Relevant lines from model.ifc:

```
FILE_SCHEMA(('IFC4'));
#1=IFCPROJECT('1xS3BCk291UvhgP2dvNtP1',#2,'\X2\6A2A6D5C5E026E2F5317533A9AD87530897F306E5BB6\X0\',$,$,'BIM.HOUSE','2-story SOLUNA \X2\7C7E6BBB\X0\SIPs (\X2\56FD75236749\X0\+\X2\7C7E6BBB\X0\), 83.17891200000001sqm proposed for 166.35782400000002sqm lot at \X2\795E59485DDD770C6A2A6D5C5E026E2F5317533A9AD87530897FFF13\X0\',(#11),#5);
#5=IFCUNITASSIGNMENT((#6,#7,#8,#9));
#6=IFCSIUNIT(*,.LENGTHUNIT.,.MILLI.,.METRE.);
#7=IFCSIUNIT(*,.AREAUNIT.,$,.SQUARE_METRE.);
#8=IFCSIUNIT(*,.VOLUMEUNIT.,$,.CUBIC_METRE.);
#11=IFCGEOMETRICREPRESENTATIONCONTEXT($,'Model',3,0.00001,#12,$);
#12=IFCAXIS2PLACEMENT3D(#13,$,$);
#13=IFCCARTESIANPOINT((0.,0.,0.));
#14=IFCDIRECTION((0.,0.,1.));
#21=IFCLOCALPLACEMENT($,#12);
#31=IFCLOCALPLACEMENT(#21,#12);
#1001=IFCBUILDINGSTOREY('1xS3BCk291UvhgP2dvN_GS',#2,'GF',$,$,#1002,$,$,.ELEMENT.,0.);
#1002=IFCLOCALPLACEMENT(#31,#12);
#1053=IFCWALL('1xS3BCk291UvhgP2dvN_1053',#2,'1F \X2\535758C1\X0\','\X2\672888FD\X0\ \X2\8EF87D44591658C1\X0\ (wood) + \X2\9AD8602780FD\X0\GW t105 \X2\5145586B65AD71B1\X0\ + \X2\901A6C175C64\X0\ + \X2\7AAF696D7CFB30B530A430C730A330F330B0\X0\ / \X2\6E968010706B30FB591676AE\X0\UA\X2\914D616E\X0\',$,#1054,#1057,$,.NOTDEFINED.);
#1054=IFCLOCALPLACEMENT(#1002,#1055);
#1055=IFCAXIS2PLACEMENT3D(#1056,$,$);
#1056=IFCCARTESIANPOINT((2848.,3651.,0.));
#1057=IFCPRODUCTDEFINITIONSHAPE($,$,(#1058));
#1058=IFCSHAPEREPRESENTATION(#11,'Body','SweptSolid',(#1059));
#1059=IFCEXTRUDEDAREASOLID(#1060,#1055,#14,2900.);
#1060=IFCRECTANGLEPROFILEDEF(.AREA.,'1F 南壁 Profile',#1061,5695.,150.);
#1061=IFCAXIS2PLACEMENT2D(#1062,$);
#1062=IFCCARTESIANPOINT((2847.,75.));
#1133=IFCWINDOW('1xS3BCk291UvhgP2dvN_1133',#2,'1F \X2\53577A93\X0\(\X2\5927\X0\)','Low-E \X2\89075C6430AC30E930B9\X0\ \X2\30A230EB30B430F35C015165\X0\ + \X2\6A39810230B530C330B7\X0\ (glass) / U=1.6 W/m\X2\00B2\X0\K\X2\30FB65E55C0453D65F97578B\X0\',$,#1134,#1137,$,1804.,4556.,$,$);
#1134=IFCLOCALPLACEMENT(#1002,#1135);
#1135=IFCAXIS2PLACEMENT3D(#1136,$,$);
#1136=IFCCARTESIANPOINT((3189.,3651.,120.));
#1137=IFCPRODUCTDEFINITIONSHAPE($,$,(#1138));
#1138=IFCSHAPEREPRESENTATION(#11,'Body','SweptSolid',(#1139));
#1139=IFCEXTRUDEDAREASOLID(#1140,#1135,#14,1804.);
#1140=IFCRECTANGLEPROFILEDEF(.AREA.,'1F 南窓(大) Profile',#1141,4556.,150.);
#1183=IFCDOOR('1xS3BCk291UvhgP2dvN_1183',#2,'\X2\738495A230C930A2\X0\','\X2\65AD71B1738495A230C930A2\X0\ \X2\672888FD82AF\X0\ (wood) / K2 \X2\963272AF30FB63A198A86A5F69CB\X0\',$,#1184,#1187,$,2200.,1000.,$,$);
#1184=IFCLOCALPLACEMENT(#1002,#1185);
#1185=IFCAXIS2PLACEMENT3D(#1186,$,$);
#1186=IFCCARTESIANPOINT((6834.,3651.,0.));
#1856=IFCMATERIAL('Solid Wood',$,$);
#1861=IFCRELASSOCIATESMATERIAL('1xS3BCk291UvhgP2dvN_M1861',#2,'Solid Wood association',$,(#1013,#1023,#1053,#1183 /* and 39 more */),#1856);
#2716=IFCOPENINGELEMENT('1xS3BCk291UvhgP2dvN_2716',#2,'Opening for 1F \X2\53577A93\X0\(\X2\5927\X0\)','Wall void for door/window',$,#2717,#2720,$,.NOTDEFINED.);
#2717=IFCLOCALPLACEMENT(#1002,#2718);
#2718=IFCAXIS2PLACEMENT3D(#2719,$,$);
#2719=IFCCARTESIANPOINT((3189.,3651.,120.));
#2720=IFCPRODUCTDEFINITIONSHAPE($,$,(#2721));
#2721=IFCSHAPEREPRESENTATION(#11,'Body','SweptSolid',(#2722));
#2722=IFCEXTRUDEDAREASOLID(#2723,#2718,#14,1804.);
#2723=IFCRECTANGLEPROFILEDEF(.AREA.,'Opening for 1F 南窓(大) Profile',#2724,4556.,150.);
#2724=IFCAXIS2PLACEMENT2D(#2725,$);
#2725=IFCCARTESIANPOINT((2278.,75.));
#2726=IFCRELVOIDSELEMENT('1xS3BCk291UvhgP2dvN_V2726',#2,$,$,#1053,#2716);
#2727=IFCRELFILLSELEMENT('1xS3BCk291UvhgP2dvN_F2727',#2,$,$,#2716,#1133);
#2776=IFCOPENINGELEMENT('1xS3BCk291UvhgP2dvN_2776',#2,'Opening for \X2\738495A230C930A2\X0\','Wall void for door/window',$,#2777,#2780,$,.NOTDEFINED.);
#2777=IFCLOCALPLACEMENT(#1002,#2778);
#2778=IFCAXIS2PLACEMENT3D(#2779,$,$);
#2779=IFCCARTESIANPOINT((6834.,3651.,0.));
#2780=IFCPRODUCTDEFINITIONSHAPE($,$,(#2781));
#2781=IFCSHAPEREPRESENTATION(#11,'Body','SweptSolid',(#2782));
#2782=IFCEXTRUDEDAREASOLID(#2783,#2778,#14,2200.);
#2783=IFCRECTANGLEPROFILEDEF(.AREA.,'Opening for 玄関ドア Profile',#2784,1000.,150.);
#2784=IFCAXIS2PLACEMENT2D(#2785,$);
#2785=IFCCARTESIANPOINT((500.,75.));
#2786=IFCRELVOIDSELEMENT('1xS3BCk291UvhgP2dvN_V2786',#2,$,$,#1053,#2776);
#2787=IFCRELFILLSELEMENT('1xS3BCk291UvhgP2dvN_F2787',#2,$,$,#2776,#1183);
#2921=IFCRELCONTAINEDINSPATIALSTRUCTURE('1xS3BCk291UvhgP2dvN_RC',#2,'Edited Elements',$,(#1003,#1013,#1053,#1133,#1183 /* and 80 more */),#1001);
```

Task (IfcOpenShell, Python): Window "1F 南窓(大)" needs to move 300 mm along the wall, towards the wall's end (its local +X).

```python
import ifcopenshell
import ifcopenshell.api.geometry
import ifcopenshell.util.placement
import ifcopenshell.util.unit

model = ifcopenshell.open("model.ifc")
unit_scale = ifcopenshell.util.unit.calculate_unit_scale(model)

window = model.by_id(1133)
opening = window.FillsVoids[0].RelatingOpeningElement
wall = opening.VoidsElements[0].RelatingBuildingElement

wall_matrix = ifcopenshell.util.placement.get_local_placement(wall.ObjectPlacement)
shift = wall_matrix[:3, 0] * 0.3 / unit_scale
before = ifcopenshell.util.placement.get_local_placement(window.ObjectPlacement)[:3, 3].copy()

# The window is not placed relative to its opening, so move both.
for product in (opening, window):
    matrix = ifcopenshell.util.placement.get_local_placement(product.ObjectPlacement)
    matrix[:3, 3] += shift
    ifcopenshell.api.geometry.edit_object_placement(model, product=product, matrix=matrix, is_si=False)

after = ifcopenshell.util.placement.get_local_placement(window.ObjectPlacement)[:3, 3]
print("window moved by", (after - before).round(3) + 0.0)

model.write("model-out.ifc")
```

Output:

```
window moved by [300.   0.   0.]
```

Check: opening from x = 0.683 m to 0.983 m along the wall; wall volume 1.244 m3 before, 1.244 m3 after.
